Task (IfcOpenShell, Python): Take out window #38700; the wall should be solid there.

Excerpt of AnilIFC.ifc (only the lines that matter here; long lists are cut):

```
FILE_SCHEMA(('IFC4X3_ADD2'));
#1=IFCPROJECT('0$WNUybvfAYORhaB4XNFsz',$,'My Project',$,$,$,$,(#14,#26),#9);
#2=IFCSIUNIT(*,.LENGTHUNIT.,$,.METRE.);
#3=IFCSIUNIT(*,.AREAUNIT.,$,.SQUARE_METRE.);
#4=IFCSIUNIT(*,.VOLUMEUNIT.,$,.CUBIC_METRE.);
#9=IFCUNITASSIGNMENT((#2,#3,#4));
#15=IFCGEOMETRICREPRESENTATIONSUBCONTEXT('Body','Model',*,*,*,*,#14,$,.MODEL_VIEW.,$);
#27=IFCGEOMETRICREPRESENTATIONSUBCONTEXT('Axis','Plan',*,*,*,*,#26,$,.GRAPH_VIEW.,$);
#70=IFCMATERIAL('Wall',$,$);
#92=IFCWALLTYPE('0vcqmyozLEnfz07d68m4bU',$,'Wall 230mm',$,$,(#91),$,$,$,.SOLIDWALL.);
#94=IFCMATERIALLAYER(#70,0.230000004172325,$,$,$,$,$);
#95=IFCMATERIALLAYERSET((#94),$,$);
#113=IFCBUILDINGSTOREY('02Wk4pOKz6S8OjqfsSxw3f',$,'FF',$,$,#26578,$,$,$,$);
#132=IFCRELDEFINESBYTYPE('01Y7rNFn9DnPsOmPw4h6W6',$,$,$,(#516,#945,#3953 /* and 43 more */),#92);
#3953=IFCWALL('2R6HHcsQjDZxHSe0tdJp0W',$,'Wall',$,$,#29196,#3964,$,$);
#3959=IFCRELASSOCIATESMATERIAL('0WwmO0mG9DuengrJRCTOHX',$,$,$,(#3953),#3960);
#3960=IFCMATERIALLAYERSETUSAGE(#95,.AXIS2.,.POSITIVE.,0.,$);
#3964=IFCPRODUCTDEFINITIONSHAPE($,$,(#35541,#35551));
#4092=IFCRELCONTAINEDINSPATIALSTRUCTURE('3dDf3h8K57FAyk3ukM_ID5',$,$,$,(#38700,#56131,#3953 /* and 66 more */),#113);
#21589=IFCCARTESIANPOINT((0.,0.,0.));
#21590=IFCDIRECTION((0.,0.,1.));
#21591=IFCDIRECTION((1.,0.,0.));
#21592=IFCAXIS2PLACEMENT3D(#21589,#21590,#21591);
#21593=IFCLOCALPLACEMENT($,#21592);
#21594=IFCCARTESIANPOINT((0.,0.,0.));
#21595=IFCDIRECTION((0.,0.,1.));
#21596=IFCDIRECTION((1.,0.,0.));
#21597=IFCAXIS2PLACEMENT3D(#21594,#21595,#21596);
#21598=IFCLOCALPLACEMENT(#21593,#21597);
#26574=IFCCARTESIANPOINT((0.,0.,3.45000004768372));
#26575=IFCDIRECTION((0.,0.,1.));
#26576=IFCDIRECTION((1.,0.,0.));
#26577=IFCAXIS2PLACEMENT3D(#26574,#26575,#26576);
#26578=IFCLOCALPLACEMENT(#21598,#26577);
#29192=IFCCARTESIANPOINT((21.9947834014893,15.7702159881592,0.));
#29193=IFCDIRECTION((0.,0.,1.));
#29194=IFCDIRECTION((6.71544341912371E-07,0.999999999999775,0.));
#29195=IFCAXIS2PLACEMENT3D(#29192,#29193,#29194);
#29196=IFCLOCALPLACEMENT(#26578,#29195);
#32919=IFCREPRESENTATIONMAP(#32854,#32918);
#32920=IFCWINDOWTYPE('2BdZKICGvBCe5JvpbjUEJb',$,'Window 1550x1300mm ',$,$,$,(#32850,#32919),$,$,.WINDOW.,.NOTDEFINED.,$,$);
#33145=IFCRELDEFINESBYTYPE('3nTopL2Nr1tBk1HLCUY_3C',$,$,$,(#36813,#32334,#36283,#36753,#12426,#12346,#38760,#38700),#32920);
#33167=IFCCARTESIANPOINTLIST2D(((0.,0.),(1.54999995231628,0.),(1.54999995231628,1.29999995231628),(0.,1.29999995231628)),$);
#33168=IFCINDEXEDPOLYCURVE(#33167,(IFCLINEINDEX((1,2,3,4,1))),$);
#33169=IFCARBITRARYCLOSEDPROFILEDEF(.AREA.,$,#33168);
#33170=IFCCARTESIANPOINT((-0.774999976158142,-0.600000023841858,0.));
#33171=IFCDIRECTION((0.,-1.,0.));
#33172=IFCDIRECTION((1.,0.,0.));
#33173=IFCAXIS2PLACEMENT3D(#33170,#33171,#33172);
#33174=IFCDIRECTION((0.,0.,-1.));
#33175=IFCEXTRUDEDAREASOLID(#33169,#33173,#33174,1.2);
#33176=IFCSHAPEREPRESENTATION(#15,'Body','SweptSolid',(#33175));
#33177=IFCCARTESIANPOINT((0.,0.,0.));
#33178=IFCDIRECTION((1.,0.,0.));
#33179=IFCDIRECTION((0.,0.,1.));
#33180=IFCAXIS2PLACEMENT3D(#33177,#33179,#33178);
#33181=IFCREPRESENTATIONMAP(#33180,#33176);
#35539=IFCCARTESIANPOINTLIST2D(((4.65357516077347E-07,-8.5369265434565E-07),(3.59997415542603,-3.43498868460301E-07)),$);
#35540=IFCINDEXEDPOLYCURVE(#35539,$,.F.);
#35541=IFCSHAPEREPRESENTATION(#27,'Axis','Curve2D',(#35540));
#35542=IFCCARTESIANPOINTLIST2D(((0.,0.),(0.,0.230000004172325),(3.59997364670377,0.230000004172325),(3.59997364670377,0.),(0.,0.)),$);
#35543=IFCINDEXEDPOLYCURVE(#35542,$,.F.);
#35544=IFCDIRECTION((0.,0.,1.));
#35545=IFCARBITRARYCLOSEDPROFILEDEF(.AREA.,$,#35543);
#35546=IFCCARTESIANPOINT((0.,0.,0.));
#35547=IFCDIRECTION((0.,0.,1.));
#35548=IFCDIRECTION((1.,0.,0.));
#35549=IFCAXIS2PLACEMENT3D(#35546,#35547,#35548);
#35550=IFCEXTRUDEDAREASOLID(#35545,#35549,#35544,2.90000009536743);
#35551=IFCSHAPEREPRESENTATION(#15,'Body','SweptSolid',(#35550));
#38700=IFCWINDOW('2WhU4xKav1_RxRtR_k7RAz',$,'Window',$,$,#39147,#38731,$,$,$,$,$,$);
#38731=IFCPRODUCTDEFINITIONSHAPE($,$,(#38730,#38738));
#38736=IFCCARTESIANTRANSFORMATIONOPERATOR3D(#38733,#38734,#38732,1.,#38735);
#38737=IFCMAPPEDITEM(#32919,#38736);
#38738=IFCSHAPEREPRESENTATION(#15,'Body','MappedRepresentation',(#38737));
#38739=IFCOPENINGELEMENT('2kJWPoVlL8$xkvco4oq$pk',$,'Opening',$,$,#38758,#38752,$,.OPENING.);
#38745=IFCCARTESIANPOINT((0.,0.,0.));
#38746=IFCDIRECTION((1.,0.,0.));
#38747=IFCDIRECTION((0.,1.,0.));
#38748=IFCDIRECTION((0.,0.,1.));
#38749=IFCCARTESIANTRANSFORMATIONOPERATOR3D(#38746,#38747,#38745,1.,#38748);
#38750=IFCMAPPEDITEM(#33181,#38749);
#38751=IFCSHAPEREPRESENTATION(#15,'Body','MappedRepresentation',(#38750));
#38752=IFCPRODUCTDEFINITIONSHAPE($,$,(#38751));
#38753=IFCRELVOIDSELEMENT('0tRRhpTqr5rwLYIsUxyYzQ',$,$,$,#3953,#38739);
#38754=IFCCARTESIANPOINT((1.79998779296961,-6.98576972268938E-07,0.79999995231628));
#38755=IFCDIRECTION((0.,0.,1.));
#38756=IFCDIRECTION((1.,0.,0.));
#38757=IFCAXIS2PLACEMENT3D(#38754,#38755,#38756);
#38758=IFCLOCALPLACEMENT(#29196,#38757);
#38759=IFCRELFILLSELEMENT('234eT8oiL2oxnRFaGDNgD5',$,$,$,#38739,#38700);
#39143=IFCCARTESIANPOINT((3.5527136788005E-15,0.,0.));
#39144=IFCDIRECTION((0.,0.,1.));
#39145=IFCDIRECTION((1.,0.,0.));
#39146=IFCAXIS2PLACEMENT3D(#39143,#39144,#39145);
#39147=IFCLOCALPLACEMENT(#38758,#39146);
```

```python
import ifcopenshell
import ifcopenshell.api.feature
import ifcopenshell.api.root
import ifcopenshell.geom
import ifcopenshell.util.shape

model = ifcopenshell.open("AnilIFC.ifc")
settings = ifcopenshell.geom.settings()


def volume(element):
    """Net volume in cubic metres, openings subtracted."""
    shape = ifcopenshell.geom.create_shape(settings, element)
    return ifcopenshell.util.shape.get_volume(shape.geometry)


window = model.by_guid("2WhU4xKav1_RxRtR_k7RAz")
opening = window.FillsVoids[0].RelatingOpeningElement
wall = opening.VoidsElements[0].RelatingBuildingElement
before = volume(wall)

ifcopenshell.api.root.remove_product(model, product=window)
ifcopenshell.api.feature.remove_feature(model, feature=opening)

after = volume(wall)

print(f"wall volume {before:.3f} -> {after:.3f} m3")

model.write("AnilIFC_edited.ifc")
```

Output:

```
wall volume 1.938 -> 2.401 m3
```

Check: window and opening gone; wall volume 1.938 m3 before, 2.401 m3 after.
